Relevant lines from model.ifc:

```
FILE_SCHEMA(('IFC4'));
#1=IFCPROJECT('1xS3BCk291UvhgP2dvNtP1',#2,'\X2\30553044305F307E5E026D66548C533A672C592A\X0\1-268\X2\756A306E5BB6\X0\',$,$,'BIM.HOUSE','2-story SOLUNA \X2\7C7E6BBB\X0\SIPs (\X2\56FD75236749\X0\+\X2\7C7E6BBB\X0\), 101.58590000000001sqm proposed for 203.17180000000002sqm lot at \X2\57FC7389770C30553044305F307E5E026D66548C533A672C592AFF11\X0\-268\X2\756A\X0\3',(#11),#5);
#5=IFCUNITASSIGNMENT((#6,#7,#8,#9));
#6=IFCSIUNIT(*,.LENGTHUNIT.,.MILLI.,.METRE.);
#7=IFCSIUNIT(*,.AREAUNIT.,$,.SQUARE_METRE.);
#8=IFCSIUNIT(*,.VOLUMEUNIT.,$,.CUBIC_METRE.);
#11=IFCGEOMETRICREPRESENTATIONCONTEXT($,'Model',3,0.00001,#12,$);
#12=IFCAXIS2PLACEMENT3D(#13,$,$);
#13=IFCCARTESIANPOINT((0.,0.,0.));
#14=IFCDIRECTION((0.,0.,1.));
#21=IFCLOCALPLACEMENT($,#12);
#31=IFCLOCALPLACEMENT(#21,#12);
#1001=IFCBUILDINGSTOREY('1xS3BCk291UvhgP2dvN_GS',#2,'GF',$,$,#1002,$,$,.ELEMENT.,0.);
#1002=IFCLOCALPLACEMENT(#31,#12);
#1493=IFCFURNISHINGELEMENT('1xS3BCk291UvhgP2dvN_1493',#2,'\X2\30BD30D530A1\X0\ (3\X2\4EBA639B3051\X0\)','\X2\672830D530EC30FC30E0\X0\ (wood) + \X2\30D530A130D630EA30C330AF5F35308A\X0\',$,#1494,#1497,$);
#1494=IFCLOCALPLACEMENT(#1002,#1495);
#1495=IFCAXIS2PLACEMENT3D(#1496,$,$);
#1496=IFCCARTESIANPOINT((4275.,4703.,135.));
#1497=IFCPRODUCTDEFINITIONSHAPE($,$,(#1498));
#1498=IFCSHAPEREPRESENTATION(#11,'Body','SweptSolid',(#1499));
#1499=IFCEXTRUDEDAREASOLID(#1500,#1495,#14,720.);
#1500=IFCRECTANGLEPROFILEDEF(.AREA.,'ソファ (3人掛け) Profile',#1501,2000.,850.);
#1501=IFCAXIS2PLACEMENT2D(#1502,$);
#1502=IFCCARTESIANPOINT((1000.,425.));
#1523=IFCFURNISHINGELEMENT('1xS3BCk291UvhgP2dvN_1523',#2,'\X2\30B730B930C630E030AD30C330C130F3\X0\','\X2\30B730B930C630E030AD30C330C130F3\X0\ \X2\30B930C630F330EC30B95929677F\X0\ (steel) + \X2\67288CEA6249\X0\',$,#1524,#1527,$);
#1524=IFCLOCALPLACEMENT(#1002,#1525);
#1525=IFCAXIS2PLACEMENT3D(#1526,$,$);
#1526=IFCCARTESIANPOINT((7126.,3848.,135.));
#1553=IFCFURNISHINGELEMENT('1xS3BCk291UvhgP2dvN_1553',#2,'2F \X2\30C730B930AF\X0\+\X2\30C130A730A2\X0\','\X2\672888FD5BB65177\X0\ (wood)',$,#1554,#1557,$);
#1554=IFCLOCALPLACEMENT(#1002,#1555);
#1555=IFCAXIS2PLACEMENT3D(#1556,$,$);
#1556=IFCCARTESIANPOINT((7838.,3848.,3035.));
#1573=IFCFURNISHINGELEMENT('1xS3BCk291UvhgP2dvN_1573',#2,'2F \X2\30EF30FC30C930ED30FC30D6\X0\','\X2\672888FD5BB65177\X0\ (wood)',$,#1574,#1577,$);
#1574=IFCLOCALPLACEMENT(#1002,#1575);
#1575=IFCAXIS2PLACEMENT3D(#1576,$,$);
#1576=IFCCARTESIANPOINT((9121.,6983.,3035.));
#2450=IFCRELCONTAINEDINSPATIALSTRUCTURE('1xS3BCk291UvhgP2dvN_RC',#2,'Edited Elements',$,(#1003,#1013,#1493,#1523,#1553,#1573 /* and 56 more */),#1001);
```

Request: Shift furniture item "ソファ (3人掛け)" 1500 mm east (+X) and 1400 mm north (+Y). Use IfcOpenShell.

```python
import ifcopenshell
import ifcopenshell.api.geometry
import ifcopenshell.util.placement
import ifcopenshell.util.unit

model = ifcopenshell.open("model.ifc")
unit_scale = ifcopenshell.util.unit.calculate_unit_scale(model)

item = model.by_guid("1xS3BCk291UvhgP2dvN_1493")
matrix = ifcopenshell.util.placement.get_local_placement(item.ObjectPlacement)
matrix[0, 3] += 1.5 / unit_scale
matrix[1, 3] += 1.4 / unit_scale
ifcopenshell.api.geometry.edit_object_placement(model, product=item, matrix=matrix, is_si=False)

print(ifcopenshell.util.placement.get_local_placement(item.ObjectPlacement).round(3) + 0.0)

model.write("model_updated.ifc")
```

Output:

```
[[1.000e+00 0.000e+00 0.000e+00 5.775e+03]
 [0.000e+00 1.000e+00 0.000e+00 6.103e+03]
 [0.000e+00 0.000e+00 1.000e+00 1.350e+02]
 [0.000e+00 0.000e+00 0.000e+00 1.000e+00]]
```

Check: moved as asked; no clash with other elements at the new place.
